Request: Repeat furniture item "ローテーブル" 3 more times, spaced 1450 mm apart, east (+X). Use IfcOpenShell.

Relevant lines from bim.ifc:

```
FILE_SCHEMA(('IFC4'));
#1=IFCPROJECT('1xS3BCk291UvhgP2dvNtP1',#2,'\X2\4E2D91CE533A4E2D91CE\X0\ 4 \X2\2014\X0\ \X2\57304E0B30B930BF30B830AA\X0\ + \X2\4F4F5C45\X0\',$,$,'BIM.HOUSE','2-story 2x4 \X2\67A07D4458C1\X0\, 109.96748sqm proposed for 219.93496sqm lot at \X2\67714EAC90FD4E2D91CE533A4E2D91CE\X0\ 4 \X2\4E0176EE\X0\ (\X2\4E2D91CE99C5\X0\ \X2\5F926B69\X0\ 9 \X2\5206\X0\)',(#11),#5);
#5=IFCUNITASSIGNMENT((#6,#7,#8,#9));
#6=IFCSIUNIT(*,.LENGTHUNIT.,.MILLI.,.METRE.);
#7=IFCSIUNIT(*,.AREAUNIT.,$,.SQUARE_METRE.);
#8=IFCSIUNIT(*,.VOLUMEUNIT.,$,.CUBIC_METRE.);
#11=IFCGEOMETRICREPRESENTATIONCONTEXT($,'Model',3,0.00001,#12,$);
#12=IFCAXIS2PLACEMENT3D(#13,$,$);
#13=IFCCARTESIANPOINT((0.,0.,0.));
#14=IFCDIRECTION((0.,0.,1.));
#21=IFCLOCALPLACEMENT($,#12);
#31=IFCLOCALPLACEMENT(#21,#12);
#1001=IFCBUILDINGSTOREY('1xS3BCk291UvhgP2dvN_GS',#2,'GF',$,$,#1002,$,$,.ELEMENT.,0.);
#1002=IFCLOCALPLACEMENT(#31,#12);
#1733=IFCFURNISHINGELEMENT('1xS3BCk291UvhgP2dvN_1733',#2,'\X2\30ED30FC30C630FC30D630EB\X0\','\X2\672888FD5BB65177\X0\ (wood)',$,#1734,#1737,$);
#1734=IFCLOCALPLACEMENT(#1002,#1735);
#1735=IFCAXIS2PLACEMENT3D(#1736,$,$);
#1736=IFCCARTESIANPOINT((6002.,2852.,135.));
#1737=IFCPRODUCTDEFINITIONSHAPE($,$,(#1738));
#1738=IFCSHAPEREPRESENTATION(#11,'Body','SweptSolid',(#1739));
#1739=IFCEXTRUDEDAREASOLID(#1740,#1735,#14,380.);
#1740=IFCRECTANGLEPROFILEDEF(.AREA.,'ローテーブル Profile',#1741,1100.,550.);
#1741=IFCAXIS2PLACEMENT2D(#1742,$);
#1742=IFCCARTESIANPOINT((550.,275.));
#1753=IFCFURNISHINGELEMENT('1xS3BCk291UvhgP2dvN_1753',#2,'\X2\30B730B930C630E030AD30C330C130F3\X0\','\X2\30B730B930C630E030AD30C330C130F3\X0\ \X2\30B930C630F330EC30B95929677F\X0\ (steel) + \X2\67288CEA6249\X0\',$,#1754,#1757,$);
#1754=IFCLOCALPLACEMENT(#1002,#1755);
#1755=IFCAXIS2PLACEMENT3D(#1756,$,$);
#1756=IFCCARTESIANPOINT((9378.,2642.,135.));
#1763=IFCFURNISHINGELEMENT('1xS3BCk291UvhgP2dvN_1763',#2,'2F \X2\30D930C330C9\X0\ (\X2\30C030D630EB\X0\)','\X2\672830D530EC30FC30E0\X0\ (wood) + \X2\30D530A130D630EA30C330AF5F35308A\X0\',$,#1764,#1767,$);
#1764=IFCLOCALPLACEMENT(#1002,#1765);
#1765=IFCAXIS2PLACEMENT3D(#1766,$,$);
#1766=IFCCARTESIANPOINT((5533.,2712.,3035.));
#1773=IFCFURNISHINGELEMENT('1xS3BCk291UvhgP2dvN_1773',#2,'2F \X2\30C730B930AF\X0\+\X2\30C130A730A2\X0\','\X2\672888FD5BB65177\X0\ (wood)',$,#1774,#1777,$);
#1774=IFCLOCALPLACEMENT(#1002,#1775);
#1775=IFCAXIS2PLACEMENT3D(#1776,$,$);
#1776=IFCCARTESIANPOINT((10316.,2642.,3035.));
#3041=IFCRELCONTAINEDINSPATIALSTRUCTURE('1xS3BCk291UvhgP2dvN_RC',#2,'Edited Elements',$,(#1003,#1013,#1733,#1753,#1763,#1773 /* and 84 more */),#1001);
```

```python
import numpy as np
import ifcopenshell
import ifcopenshell.api.geometry
import ifcopenshell.api.root
import ifcopenshell.util.element
import ifcopenshell.util.placement

model = ifcopenshell.open("bim.ifc")


def reuse_history(source, copy):
    """copy_class also copies each property set's owner history, people and application; keep the originals."""
    for rel in copy.IsDefinedBy:
        if rel.is_a("IfcRelDefinesByProperties") and (history := rel.RelatingPropertyDefinition.OwnerHistory):
            rel.RelatingPropertyDefinition.OwnerHistory = source.OwnerHistory
            ifcopenshell.util.element.remove_deep2(model, history)


source = model.by_id(1733)
base = ifcopenshell.util.placement.get_local_placement(source.ObjectPlacement)
step = np.array([1.0, 0.0, 0.0]) * 1450.0

for i in range(1, 4):
    copy = ifcopenshell.api.root.copy_class(model, product=source)
    copy.Representation = ifcopenshell.util.element.copy_deep(
        model, source.Representation, exclude=["IfcGeometricRepresentationContext", "IfcRepresentationMap"]
    )
    reuse_history(source, copy)
    matrix = base.copy()
    matrix[:3, 3] += i * step
    print("added at", matrix[:3, 3].round(3) + 0.0)
    ifcopenshell.api.geometry.edit_object_placement(model, product=copy, matrix=matrix, is_si=False)

model.write("bim_edited.ifc")
```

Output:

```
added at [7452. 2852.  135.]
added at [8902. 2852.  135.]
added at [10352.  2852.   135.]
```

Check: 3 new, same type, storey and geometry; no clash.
